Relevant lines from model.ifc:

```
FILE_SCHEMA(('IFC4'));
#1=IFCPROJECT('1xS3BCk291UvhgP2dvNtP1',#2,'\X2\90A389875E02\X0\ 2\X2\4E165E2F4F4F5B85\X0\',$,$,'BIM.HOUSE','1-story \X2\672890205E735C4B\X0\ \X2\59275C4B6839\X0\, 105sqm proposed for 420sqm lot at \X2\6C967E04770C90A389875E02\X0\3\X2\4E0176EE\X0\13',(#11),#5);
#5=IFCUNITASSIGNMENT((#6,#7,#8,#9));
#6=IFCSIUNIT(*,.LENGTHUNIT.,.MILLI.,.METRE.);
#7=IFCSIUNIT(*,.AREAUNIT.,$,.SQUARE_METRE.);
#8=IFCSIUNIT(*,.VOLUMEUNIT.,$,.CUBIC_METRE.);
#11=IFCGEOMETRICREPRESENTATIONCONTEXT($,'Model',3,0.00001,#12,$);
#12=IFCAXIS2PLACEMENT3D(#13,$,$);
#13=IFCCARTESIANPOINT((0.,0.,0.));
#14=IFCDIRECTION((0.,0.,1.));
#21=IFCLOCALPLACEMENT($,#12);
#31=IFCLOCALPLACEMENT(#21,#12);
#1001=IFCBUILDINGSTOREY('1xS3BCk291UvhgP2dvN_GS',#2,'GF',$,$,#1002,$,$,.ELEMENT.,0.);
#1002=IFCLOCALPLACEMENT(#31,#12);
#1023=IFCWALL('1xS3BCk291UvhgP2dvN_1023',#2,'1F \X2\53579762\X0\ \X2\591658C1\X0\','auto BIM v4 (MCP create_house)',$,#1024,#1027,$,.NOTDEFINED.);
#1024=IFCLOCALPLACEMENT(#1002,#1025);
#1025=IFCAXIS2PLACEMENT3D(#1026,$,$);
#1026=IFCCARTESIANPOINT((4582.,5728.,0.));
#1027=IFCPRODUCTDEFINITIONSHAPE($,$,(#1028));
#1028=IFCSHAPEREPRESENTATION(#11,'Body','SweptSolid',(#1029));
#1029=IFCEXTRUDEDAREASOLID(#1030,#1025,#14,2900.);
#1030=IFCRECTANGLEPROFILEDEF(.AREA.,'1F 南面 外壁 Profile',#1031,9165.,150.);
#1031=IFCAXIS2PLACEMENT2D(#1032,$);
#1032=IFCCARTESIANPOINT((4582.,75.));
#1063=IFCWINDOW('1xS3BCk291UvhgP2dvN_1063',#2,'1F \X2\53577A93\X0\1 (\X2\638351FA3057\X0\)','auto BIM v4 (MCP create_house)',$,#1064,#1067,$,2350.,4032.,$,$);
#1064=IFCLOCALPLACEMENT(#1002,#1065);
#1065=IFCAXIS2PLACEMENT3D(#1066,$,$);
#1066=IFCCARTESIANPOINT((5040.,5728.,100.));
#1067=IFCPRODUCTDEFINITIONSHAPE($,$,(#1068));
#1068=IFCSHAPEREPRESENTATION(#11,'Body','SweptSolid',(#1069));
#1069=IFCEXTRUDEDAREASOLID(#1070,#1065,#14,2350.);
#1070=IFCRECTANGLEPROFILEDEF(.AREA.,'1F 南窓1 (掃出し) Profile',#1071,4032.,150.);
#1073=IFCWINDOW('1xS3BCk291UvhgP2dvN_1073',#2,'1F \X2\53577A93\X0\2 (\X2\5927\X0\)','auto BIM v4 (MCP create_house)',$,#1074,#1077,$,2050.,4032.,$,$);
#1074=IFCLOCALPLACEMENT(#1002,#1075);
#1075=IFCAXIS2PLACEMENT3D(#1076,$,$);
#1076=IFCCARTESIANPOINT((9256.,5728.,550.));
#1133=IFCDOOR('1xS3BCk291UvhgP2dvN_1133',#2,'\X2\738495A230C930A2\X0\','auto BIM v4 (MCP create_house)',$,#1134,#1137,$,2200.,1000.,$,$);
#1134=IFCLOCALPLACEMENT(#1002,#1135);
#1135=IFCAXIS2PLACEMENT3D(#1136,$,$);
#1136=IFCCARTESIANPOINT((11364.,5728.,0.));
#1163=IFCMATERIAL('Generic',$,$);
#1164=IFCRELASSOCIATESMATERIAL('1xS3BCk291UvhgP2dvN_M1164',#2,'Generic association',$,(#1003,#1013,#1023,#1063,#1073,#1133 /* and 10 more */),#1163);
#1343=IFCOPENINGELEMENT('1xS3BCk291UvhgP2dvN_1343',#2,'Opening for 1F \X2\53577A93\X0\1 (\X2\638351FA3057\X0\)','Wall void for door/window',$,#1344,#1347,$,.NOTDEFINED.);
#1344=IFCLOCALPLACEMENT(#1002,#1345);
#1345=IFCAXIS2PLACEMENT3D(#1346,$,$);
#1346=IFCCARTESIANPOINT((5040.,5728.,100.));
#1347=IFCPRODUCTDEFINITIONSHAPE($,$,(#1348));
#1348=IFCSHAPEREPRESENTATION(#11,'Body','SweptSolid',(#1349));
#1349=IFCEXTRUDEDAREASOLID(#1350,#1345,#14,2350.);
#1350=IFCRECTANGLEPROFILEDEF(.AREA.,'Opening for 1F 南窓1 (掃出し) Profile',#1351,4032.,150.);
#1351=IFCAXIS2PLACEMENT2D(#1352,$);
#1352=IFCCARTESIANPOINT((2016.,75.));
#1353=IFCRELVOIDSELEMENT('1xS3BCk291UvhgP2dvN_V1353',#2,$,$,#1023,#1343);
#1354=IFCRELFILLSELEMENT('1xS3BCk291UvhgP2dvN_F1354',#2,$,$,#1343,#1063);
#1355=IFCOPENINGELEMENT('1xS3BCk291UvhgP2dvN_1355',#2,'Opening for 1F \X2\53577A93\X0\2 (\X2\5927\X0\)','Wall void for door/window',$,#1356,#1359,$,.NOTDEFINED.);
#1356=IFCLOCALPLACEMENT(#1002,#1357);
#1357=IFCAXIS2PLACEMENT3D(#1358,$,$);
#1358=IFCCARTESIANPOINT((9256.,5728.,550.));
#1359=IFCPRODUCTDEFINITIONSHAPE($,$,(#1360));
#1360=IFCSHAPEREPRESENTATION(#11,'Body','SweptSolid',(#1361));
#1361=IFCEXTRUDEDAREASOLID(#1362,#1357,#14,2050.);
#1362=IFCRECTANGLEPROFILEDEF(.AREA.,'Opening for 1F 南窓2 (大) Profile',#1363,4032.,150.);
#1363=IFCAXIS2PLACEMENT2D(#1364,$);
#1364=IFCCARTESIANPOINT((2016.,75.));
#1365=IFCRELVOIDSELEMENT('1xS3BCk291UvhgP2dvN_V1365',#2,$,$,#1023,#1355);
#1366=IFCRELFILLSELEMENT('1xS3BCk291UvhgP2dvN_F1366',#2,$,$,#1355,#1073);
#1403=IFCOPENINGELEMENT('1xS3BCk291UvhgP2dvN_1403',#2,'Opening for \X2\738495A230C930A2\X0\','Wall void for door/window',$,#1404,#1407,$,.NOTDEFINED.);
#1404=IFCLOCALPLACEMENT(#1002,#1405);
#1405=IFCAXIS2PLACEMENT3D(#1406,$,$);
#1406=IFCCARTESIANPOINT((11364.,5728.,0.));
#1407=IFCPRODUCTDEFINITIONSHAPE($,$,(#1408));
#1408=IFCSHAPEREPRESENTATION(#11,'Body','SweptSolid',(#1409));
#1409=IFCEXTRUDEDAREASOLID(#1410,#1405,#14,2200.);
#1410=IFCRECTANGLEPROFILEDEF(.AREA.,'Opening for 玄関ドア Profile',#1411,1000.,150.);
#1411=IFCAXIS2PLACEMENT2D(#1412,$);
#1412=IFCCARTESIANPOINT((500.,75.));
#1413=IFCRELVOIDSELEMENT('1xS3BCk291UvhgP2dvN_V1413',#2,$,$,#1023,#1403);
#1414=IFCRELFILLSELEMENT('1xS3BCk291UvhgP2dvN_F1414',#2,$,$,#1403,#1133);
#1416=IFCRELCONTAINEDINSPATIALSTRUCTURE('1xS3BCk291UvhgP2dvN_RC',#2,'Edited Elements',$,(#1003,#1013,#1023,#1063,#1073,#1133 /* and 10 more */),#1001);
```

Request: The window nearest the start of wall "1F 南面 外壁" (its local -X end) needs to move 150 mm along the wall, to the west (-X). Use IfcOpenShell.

```python
import ifcopenshell
import ifcopenshell.api.geometry
import ifcopenshell.util.placement

model = ifcopenshell.open("model.ifc")

window = model.by_guid("1xS3BCk291UvhgP2dvN_1063")
opening = window.FillsVoids[0].RelatingOpeningElement
wall = opening.VoidsElements[0].RelatingBuildingElement

wall_matrix = ifcopenshell.util.placement.get_local_placement(wall.ObjectPlacement)
shift = wall_matrix[:3, 0] * -150.0
before = ifcopenshell.util.placement.get_local_placement(window.ObjectPlacement)[:3, 3].copy()

# The window is not placed relative to its opening, so move both.
for product in (opening, window):
    matrix = ifcopenshell.util.placement.get_local_placement(product.ObjectPlacement)
    matrix[:3, 3] += shift
    ifcopenshell.api.geometry.edit_object_placement(model, product=product, matrix=matrix, is_si=False)

after = ifcopenshell.util.placement.get_local_placement(window.ObjectPlacement)[:3, 3]
print("window moved by", (after - before).round(3) + 0.0)

model.write("model_updated.ifc")
```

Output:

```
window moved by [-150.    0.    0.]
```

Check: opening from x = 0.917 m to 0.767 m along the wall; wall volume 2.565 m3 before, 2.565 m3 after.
